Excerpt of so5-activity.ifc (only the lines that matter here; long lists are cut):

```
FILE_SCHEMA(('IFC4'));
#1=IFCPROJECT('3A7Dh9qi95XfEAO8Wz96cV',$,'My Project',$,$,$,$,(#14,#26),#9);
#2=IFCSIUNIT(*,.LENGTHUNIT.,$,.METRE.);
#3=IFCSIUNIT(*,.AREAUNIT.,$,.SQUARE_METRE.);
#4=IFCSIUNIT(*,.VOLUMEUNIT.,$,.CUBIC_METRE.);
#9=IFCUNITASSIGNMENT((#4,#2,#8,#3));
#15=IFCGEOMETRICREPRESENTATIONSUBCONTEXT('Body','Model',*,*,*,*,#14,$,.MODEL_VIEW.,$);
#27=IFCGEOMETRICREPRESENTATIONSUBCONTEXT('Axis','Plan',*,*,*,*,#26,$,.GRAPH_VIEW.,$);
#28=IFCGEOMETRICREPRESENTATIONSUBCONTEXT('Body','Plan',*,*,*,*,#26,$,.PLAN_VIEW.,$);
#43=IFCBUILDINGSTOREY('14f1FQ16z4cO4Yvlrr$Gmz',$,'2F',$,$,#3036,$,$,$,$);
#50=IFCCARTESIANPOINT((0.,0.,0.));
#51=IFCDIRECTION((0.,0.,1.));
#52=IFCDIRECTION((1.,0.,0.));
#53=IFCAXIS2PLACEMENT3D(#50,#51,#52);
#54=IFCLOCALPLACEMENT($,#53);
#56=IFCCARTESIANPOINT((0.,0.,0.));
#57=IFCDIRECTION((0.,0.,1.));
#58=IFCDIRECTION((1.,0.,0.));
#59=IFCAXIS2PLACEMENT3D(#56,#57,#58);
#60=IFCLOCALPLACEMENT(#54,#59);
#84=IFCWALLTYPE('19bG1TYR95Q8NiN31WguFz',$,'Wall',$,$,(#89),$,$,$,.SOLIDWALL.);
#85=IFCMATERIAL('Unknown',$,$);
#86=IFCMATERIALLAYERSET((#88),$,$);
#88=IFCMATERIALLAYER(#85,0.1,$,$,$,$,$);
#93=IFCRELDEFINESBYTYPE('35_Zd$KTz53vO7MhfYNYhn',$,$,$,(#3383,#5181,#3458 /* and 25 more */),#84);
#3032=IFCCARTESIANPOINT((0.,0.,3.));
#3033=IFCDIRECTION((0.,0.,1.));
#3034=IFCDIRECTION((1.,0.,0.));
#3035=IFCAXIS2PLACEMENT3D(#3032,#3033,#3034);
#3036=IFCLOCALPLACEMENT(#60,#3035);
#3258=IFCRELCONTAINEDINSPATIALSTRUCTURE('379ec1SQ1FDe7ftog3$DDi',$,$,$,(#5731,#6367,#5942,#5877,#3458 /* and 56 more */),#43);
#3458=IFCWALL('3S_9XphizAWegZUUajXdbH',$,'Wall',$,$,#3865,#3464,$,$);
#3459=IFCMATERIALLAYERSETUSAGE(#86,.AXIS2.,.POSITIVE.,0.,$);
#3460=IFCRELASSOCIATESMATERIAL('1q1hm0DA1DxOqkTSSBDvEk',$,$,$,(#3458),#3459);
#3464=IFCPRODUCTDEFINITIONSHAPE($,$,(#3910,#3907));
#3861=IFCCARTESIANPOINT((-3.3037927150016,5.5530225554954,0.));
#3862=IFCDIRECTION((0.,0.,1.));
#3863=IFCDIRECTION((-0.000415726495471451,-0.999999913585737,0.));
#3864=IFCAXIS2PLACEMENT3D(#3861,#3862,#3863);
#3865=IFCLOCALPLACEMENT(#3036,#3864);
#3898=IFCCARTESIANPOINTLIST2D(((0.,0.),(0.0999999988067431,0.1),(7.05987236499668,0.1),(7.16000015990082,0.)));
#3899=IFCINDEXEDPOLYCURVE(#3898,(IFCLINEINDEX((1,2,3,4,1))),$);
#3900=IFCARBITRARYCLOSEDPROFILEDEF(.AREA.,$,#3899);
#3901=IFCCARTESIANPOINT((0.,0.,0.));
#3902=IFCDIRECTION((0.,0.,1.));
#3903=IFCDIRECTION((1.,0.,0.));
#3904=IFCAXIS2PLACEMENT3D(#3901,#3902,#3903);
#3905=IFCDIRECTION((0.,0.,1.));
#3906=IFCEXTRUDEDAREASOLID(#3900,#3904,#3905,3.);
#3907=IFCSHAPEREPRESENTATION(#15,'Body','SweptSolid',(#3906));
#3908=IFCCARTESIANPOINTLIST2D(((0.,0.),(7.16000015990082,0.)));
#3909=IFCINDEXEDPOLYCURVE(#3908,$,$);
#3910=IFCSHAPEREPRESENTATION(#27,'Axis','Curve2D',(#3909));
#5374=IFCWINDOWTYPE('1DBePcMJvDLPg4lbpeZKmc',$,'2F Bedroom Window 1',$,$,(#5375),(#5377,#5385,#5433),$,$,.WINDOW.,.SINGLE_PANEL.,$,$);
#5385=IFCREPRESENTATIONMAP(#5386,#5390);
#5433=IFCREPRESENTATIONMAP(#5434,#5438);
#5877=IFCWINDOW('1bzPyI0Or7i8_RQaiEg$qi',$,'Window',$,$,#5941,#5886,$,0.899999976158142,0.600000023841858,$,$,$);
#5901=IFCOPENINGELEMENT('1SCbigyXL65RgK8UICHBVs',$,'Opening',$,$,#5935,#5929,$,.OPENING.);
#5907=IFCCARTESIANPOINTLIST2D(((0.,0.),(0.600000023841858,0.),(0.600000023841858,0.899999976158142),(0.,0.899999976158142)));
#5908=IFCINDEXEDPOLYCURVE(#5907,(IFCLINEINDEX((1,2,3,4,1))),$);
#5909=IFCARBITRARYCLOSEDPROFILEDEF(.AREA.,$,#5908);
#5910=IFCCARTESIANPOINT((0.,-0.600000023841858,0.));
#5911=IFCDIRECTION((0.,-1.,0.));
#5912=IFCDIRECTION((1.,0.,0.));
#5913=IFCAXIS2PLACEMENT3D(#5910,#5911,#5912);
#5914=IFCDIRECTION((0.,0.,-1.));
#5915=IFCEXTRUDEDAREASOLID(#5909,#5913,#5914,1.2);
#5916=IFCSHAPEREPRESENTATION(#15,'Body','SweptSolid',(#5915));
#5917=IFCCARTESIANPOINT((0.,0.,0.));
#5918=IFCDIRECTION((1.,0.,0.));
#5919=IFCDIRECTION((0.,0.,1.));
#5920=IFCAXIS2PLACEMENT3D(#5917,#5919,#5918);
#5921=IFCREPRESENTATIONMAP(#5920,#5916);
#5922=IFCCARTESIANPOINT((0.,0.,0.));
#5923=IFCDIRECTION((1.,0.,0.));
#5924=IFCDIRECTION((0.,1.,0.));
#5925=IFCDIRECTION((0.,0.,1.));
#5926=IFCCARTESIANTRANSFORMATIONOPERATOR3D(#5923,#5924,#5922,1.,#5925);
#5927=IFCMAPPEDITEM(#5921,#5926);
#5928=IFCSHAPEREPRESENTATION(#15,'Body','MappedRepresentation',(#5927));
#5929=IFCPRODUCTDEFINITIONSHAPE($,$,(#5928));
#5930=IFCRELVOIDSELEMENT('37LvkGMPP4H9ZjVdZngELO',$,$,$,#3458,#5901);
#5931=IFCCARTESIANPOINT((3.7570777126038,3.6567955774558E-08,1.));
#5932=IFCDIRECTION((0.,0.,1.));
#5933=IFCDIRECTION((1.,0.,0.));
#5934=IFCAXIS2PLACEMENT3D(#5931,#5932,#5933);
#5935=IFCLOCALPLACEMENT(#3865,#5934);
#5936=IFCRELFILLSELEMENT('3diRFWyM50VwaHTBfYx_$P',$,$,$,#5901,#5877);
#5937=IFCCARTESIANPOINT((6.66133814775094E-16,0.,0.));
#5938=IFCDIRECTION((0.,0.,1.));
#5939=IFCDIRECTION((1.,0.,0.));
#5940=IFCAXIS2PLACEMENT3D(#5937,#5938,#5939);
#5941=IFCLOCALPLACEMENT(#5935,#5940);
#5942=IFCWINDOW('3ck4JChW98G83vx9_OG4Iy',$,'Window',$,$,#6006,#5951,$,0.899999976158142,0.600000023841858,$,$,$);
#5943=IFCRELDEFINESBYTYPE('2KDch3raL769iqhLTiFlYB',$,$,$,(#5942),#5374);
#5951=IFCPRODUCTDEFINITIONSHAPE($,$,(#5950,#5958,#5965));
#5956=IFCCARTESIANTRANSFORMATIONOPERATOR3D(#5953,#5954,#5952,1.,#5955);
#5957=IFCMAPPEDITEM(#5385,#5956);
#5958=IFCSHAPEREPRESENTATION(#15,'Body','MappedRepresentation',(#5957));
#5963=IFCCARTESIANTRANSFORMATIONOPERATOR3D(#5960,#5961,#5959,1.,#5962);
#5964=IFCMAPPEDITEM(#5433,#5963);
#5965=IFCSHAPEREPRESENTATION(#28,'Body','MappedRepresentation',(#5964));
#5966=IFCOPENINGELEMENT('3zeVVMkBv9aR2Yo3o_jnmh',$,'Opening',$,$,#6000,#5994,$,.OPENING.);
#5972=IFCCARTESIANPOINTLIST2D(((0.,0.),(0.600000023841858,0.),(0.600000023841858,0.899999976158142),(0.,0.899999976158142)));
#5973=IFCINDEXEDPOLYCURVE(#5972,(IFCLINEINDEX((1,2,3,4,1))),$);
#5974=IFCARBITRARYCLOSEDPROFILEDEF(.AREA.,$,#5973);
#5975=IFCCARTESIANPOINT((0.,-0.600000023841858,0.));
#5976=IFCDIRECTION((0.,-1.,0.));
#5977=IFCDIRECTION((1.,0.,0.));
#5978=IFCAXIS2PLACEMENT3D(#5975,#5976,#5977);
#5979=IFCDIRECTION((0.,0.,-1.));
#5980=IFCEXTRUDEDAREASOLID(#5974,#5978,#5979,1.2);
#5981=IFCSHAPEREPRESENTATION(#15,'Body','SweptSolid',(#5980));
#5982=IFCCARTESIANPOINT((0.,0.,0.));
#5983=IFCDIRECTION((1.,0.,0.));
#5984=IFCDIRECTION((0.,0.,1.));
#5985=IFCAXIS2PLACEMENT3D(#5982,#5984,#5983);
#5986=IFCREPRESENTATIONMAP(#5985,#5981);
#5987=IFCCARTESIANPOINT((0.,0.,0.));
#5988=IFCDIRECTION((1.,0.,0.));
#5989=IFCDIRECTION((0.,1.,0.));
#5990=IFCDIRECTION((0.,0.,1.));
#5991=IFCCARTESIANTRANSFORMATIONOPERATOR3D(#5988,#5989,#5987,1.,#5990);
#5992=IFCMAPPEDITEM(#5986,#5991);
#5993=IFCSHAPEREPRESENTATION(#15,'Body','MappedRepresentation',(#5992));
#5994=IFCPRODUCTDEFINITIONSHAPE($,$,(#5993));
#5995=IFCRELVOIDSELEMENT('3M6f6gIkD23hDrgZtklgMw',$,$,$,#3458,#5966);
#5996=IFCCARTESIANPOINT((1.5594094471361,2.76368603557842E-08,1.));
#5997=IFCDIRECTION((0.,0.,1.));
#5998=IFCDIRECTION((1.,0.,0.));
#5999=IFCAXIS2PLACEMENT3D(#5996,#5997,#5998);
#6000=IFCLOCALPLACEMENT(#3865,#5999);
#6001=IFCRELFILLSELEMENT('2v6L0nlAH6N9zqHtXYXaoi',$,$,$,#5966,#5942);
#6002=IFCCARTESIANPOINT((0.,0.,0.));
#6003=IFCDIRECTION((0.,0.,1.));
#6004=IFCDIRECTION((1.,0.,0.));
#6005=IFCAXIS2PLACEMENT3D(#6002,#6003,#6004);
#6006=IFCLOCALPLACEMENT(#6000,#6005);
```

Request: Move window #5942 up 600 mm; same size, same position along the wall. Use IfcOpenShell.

```python
import numpy as np
import ifcopenshell
import ifcopenshell.api.geometry
import ifcopenshell.util.placement
import ifcopenshell.util.unit

model = ifcopenshell.open("so5-activity.ifc")
unit_scale = ifcopenshell.util.unit.calculate_unit_scale(model)

window = model.by_guid("3ck4JChW98G83vx9_OG4Iy")
opening = window.FillsVoids[0].RelatingOpeningElement
dz = 0.6 / unit_scale

shift = np.array([0.0, 0.0, dz])
# The window is placed relative to its opening, so it follows when the opening moves.
matrix = ifcopenshell.util.placement.get_local_placement(opening.ObjectPlacement)
matrix[:3, 3] += shift
ifcopenshell.api.geometry.edit_object_placement(
    model, product=opening, matrix=matrix, is_si=False, should_transform_children=True
)

print(f"moved by {dz * unit_scale:+.3f} m")

model.write("so5-activity_updated.ifc")
```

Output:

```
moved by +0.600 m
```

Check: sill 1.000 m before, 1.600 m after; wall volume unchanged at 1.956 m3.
